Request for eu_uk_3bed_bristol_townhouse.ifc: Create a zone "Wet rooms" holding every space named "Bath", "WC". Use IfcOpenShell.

First a look at what the model holds.

```python
import ifcopenshell

model = ifcopenshell.open("eu_uk_3bed_bristol_townhouse.ifc")
print(model.schema)
seen = {}
for space in model.by_type("IfcSpace"):
    seen[space.LongName] = seen.get(space.LongName, 0) + 1
for name, count in sorted(seen.items(), key=str):
    print(count, "x", name)
print("zones:", [z.Name for z in model.by_type("IfcZone")][:20])
```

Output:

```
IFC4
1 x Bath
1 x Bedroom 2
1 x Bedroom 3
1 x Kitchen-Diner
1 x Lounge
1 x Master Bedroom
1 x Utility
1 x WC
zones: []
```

```python
import ifcopenshell
import ifcopenshell.api.group
import ifcopenshell.api.root

model = ifcopenshell.open("eu_uk_3bed_bristol_townhouse.ifc")

names = {"Bath", "WC"}
spaces = [s for s in model.by_type("IfcSpace") if s.LongName in names]

zone = ifcopenshell.api.root.create_entity(model, ifc_class="IfcZone", name="Wet rooms")
ifcopenshell.api.group.assign_group(model, products=spaces, group=zone)
print(len(spaces), "spaces in", zone.Name)

model.write("eu_uk_3bed_bristol_townhouse_rev.ifc")
```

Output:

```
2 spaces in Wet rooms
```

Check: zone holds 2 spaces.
